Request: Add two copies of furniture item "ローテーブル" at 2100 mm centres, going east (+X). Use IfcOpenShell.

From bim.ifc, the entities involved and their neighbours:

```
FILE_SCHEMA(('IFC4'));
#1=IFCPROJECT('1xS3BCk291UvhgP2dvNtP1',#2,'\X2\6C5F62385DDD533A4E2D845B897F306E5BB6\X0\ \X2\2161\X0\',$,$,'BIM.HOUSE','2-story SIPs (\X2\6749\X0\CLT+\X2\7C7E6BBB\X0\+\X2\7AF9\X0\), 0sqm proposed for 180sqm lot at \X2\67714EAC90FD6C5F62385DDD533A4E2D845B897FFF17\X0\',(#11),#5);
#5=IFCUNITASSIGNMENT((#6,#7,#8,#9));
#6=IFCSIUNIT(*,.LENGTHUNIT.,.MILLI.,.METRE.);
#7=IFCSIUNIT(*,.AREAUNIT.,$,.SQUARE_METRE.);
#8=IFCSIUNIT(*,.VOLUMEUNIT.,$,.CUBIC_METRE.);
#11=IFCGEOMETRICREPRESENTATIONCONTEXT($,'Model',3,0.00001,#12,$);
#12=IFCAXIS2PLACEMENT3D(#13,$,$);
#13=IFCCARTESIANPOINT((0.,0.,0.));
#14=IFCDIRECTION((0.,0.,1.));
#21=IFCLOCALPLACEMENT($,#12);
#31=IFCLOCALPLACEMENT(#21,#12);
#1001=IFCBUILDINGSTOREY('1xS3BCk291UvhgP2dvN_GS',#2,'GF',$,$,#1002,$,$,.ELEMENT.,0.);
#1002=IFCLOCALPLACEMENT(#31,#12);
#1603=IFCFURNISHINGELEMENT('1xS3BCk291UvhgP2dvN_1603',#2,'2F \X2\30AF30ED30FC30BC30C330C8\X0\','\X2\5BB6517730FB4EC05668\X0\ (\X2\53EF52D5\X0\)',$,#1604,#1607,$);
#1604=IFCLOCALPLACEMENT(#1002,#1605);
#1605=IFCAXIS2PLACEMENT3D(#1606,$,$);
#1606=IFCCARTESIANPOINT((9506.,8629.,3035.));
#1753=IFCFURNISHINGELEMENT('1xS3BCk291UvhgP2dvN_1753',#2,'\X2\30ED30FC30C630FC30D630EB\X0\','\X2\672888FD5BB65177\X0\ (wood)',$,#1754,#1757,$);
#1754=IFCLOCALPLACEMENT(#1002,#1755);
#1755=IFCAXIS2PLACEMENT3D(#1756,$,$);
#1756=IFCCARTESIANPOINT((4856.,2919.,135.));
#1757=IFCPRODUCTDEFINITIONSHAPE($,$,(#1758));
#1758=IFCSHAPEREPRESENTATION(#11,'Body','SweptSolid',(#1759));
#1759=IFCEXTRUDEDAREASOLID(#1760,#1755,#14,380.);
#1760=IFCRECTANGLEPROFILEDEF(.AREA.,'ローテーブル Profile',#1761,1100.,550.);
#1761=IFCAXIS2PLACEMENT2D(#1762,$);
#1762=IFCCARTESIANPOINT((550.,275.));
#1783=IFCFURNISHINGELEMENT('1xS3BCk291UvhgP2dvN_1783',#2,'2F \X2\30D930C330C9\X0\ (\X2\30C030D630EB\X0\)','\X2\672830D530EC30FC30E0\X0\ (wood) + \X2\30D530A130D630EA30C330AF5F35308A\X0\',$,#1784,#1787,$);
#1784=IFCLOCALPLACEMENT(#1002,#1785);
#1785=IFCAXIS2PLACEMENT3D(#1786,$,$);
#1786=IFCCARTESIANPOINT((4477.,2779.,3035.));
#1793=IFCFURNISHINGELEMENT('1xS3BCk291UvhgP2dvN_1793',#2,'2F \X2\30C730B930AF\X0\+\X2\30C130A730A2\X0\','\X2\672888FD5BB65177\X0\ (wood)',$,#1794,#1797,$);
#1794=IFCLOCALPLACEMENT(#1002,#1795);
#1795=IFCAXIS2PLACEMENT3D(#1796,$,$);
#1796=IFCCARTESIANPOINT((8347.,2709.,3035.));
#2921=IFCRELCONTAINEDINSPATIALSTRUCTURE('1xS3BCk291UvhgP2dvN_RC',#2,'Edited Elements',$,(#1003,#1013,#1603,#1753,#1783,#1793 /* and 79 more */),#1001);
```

```python
import numpy as np
import ifcopenshell
import ifcopenshell.api.geometry
import ifcopenshell.api.root
import ifcopenshell.util.element
import ifcopenshell.util.placement

model = ifcopenshell.open("bim.ifc")


def reuse_history(source, copy):
    """copy_class also copies each property set's owner history, people and application; keep the originals."""
    for rel in copy.IsDefinedBy:
        if rel.is_a("IfcRelDefinesByProperties") and (history := rel.RelatingPropertyDefinition.OwnerHistory):
            rel.RelatingPropertyDefinition.OwnerHistory = source.OwnerHistory
            ifcopenshell.util.element.remove_deep2(model, history)


source = model.by_guid("1xS3BCk291UvhgP2dvN_1753")
base = ifcopenshell.util.placement.get_local_placement(source.ObjectPlacement)
step = np.array([1.0, 0.0, 0.0]) * 2100.0

for i in range(1, 3):
    copy = ifcopenshell.api.root.copy_class(model, product=source)
    copy.Representation = ifcopenshell.util.element.copy_deep(
        model, source.Representation, exclude=["IfcGeometricRepresentationContext", "IfcRepresentationMap"]
    )
    reuse_history(source, copy)
    matrix = base.copy()
    matrix[:3, 3] += i * step
    print("added at", matrix[:3, 3].round(3) + 0.0)
    ifcopenshell.api.geometry.edit_object_placement(model, product=copy, matrix=matrix, is_si=False)

model.write("bim_rev.ifc")
```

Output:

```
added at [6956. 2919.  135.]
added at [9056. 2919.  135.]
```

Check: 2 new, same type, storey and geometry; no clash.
